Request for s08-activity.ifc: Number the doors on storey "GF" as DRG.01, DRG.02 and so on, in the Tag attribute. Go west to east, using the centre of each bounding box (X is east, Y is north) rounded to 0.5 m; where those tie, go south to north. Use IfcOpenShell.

First a look at what the model holds.

```python
import ifcopenshell
import ifcopenshell.util.element
import ifcopenshell.util.placement

model = ifcopenshell.open("s08-activity.ifc")
print(model.schema)
storey = next(s for s in model.by_type("IfcBuildingStorey") if s.Name == "GF")
doors = [e for e in ifcopenshell.util.element.get_decomposition(storey) if e.is_a("IfcDoor")]
for e in sorted(doors, key=lambda e: e.id()):
    origin = ifcopenshell.util.placement.get_local_placement(e.ObjectPlacement)[:3, 3]
    print(e.id(), e.Tag, e.Name, origin.round(2) + 0.0, sep=" | ")
```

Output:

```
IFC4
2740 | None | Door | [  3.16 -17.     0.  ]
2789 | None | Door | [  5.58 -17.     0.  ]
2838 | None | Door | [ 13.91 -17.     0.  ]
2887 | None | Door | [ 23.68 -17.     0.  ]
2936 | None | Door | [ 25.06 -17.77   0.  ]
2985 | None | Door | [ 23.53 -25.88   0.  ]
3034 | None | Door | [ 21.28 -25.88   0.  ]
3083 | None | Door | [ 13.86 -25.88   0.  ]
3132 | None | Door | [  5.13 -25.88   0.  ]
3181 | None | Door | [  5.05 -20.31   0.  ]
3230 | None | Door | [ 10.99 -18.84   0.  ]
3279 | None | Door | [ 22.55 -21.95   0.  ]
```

```python
import ifcopenshell
import ifcopenshell.geom
import ifcopenshell.util.element
import ifcopenshell.util.shape

model = ifcopenshell.open("s08-activity.ifc")
settings = ifcopenshell.geom.settings()
settings.set("use-world-coords", True)


def centre(element):
    shape = ifcopenshell.geom.create_shape(settings, element)
    return ifcopenshell.util.shape.get_bbox_centroid(shape.geometry)


storey = next(s for s in model.by_type("IfcBuildingStorey") if s.Name == "GF")
doors = [e for e in ifcopenshell.util.element.get_decomposition(storey) if e.is_a("IfcDoor")]

# Insertion points can sit at a corner or the storey origin, so sort by the geometry (in metres).
centres = {e: centre(e) for e in doors}
doors.sort(key=lambda e: (round(centres[e][0] / 0.5), centres[e][1]))

for i, e in enumerate(doors, start=1):
    number = f"DRG.{i:02d}"
    e.Tag = number
    print(e.id(), number)

model.write("s08-activity_rev.ifc")
```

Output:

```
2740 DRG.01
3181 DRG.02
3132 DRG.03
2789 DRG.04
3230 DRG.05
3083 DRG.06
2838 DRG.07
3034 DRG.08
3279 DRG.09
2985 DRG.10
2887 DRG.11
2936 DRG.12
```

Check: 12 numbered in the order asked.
